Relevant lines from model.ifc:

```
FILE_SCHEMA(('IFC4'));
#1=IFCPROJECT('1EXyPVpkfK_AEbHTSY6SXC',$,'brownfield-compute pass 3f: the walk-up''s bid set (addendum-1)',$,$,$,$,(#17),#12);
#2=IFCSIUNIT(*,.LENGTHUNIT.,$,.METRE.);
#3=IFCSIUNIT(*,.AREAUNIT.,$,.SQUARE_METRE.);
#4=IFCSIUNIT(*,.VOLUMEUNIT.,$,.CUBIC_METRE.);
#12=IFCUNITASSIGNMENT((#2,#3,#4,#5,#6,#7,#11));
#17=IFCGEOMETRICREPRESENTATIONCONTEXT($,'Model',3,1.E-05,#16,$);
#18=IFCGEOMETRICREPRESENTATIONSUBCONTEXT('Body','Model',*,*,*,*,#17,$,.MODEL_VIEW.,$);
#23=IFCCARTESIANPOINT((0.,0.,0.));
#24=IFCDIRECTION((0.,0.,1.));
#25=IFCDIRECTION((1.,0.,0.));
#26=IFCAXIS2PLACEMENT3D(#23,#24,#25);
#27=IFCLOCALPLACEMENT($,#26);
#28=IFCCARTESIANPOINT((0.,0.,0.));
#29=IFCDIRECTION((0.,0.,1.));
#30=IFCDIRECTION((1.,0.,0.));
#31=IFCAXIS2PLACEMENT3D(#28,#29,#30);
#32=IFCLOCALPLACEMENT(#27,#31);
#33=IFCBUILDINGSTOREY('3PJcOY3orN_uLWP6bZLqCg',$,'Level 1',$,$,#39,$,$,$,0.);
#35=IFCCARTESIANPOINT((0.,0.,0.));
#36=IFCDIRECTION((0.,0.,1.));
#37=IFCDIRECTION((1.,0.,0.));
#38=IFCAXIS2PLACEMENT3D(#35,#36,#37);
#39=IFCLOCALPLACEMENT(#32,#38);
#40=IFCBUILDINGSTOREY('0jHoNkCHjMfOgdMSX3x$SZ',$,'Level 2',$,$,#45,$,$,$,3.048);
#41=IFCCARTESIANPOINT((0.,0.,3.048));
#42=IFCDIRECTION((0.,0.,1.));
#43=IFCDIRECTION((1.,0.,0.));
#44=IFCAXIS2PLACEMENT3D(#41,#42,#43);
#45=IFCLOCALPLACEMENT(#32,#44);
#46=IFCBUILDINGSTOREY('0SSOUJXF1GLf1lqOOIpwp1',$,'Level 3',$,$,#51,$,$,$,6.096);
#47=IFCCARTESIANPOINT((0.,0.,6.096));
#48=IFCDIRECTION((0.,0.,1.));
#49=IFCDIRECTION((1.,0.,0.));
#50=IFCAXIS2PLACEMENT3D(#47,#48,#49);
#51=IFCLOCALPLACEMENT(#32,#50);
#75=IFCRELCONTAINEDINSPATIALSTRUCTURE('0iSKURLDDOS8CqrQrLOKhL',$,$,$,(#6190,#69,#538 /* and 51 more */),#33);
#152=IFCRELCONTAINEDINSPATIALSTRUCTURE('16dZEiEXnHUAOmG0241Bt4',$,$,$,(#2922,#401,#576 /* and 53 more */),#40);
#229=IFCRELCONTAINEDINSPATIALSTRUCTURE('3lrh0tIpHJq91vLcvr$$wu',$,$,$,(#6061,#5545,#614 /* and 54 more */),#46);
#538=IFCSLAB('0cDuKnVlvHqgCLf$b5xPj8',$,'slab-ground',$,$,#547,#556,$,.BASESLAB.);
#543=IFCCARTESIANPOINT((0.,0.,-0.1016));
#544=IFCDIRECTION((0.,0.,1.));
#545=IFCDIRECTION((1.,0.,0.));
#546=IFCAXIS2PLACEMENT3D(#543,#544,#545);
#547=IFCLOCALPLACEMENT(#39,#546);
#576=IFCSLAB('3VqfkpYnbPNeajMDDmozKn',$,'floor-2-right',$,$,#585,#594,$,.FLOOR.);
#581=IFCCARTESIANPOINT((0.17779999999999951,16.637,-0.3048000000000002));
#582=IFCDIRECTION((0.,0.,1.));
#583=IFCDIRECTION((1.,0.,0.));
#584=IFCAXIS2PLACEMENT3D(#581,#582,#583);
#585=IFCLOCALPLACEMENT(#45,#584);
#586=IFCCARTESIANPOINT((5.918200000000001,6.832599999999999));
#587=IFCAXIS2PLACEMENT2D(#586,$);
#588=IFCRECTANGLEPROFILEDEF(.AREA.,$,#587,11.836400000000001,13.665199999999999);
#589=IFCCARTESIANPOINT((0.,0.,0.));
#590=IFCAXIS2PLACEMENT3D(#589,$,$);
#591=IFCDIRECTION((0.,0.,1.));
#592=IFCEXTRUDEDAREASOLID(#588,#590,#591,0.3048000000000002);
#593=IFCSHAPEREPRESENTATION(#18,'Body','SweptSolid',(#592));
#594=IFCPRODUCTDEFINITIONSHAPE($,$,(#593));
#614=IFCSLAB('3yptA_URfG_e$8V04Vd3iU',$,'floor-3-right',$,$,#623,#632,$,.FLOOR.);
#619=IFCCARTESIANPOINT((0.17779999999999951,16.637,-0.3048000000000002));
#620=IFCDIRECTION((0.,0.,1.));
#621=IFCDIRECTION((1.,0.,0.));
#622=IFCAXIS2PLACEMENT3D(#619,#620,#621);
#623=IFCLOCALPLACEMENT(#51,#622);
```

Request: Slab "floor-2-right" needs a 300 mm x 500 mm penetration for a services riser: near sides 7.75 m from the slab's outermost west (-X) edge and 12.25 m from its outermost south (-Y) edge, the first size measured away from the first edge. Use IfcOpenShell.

```python
import numpy as np
import ifcopenshell
import ifcopenshell.api.feature
import ifcopenshell.api.geometry
import ifcopenshell.api.root
import ifcopenshell.geom
import ifcopenshell.util.placement
import ifcopenshell.util.representation
import ifcopenshell.util.shape
import ifcopenshell.util.unit

model = ifcopenshell.open("model.ifc")
unit_scale = ifcopenshell.util.unit.calculate_unit_scale(model)
settings = ifcopenshell.geom.settings()


def volume(element):
    """Net volume in cubic metres, openings subtracted."""
    shape = ifcopenshell.geom.create_shape(settings, element)
    return ifcopenshell.util.shape.get_volume(shape.geometry)


slab = model.by_guid("3VqfkpYnbPNeajMDDmozKn")
before = volume(slab)

# Extent in the slab's own axes, in metres. The edges named are its -X and -Y sides.
slab_shape = ifcopenshell.geom.create_shape(settings, slab)
vertices = ifcopenshell.util.shape.get_vertices(slab_shape.geometry)
x_min, y_min, bottom = vertices.min(axis=0)
top = vertices[:, 2].max()

opening = ifcopenshell.api.root.create_entity(model, ifc_class="IfcOpeningElement", name="Services riser opening", predefined_type="OPENING")
context = ifcopenshell.util.representation.get_context(model, "Model", "Body", "MODEL_VIEW")
width, depth = 0.3, 0.5
outline = [(0.0, 0.0), (width, 0.0), (width, depth), (0.0, depth), (0.0, 0.0)]
# Overshoot both faces by 50 mm so the cut is clean.
shape = ifcopenshell.api.geometry.add_slab_representation(
    model, context=context, depth=top - bottom + 0.1, polyline=outline
)
ifcopenshell.api.geometry.assign_representation(model, product=opening, representation=shape)

matrix = ifcopenshell.util.placement.get_local_placement(slab.ObjectPlacement)
matrix[:, 3] = matrix @ np.append(np.array([x_min + 7.75, y_min + 12.25, bottom - 0.05]) / unit_scale, 1.0)
ifcopenshell.api.geometry.edit_object_placement(model, product=opening, matrix=matrix, is_si=False)
ifcopenshell.api.feature.add_feature(model, feature=opening, element=slab)

after = volume(slab)

print(f"slab volume {before:.3f} -> {after:.3f} m3")

model.write("model_edited.ifc")
```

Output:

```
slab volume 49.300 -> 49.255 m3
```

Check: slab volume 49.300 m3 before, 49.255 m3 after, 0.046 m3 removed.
